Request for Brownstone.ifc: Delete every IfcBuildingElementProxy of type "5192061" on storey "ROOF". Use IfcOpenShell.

First a look at what the model holds.

```python
import ifcopenshell
import ifcopenshell.util.element

model = ifcopenshell.open("Brownstone.ifc")
print(model.schema)
storey = next(s for s in model.by_type("IfcBuildingStorey") if s.Name == "ROOF")
proxies = [e for e in ifcopenshell.util.element.get_decomposition(storey) if e.is_a("IfcBuildingElementProxy")]
seen = {}
for e in proxies:
    element_type = ifcopenshell.util.element.get_type(e)
    name = element_type.Name if element_type not in (None, e) else None
    seen[name] = seen.get(name, 0) + 1
for name, count in sorted(seen.items(), key=str):
    print(count, "x", name)
```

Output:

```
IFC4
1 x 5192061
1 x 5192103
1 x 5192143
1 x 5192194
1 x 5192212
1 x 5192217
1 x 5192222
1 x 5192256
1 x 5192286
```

```python
import ifcopenshell
import ifcopenshell.api.root
import ifcopenshell.util.element

model = ifcopenshell.open("Brownstone.ifc")

storey = next(s for s in model.by_type("IfcBuildingStorey") if s.Name == "ROOF")
proxies = [e for e in ifcopenshell.util.element.get_decomposition(storey) if e.is_a("IfcBuildingElementProxy")]
targets = [e for e in proxies if (t := ifcopenshell.util.element.get_type(e)) not in (None, e) and t.Name == "5192061"]

for e in targets:
    ifcopenshell.api.root.remove_product(model, product=e)
print(len(targets), "removed")

model.write("Brownstone_rev.ifc")
```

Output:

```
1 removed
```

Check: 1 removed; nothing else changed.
